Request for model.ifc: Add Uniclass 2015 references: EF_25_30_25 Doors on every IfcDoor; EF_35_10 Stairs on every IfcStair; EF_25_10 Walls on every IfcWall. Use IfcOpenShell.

First a look at what the model holds.

```python
import ifcopenshell

model = ifcopenshell.open("model.ifc")
print(model.schema)
print("classifications:", [c.Name for c in model.by_type("IfcClassification")])
for ifc_class in ("IfcDoor", "IfcRoof", "IfcStair", "IfcWall", "IfcWindow"):
    print(ifc_class, len(model.by_type(ifc_class)))
```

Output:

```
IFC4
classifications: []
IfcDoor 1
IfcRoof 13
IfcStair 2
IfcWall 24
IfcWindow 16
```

```python
import ifcopenshell
import ifcopenshell.api.classification

model = ifcopenshell.open("model.ifc")

system = ifcopenshell.api.classification.add_classification(model, classification="Uniclass 2015")

codes = {
    "IfcDoor": ("EF_25_30_25", "Doors"),
    "IfcStair": ("EF_35_10", "Stairs"),
    "IfcWall": ("EF_25_10", "Walls"),
}
for ifc_class, (code, name) in codes.items():
    products = model.by_type(ifc_class)
    ifcopenshell.api.classification.add_reference(
        model, products=products, classification=system, identification=code, name=name
    )
    print(code, len(products))

model.write("model_v2.ifc")
```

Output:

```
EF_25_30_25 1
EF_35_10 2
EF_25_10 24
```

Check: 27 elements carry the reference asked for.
